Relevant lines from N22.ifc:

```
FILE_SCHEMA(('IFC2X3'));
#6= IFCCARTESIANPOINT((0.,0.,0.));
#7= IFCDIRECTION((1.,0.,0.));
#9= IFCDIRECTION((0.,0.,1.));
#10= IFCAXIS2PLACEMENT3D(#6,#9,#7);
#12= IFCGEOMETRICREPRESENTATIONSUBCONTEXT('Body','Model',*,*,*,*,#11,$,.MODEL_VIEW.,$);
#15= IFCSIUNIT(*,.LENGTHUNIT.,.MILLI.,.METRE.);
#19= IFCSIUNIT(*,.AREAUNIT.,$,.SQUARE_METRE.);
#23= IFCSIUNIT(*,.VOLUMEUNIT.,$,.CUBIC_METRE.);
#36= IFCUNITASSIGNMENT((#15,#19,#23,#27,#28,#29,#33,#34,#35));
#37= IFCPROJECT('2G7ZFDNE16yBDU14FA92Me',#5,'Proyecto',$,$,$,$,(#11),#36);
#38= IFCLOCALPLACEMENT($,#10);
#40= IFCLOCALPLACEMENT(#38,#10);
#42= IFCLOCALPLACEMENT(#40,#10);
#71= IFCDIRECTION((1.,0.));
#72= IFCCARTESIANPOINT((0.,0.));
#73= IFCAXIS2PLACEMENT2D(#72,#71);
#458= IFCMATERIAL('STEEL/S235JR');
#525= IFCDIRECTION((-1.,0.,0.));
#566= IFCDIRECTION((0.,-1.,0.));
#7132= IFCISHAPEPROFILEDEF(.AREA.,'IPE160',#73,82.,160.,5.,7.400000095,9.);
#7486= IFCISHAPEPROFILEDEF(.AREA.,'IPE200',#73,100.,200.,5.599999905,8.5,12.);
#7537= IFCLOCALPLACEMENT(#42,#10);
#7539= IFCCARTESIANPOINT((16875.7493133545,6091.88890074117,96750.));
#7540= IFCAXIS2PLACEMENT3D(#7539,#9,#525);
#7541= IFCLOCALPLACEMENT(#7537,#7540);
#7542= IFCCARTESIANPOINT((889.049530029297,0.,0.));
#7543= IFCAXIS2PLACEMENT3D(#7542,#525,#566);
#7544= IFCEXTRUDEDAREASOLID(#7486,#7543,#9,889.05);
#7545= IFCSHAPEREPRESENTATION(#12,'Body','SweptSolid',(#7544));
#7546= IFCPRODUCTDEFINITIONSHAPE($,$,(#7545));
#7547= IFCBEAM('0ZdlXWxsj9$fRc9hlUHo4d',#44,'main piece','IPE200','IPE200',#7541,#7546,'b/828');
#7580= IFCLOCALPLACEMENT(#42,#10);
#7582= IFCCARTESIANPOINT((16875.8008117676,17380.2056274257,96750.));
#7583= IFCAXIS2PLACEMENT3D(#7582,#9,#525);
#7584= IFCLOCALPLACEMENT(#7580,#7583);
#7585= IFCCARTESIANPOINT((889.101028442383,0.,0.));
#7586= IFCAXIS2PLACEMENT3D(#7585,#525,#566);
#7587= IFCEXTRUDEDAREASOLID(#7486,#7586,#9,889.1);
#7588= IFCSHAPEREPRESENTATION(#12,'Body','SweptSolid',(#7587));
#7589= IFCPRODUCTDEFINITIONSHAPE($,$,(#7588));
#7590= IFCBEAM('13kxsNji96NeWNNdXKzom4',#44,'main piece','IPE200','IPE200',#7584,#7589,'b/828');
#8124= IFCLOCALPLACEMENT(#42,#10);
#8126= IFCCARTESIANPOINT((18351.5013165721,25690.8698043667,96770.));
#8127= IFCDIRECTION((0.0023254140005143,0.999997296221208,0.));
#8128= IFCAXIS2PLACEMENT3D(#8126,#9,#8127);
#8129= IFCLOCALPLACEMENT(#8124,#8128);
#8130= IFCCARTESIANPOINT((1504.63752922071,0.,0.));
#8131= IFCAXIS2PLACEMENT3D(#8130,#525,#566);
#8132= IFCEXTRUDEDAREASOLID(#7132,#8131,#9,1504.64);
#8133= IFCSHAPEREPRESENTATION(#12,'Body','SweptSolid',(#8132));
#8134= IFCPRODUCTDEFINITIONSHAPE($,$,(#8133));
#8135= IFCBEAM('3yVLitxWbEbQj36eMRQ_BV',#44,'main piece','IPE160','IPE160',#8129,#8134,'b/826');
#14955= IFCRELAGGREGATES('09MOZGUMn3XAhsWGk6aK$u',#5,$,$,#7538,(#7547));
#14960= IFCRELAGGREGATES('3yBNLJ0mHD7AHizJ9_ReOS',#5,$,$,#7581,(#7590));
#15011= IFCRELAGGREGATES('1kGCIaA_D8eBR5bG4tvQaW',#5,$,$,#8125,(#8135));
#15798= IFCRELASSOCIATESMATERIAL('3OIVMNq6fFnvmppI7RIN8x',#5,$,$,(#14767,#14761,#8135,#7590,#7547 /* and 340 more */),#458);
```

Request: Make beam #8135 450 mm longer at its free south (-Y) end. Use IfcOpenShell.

```python
import ifcopenshell
import ifcopenshell.util.representation

model = ifcopenshell.open("N22.ifc")

member = model.by_id(8135)
change = 450.0

# The extrusion runs towards the end named, so only its depth changes.
body = ifcopenshell.util.representation.get_representation(member, "Model", "Body")
solid = body.Items[0]
old_length = solid.Depth
solid.Depth += change

print(f"length {old_length:g} -> {solid.Depth:g}")

model.write("N22_edited.ifc")
```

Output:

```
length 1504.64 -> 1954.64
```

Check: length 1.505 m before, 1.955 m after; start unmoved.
